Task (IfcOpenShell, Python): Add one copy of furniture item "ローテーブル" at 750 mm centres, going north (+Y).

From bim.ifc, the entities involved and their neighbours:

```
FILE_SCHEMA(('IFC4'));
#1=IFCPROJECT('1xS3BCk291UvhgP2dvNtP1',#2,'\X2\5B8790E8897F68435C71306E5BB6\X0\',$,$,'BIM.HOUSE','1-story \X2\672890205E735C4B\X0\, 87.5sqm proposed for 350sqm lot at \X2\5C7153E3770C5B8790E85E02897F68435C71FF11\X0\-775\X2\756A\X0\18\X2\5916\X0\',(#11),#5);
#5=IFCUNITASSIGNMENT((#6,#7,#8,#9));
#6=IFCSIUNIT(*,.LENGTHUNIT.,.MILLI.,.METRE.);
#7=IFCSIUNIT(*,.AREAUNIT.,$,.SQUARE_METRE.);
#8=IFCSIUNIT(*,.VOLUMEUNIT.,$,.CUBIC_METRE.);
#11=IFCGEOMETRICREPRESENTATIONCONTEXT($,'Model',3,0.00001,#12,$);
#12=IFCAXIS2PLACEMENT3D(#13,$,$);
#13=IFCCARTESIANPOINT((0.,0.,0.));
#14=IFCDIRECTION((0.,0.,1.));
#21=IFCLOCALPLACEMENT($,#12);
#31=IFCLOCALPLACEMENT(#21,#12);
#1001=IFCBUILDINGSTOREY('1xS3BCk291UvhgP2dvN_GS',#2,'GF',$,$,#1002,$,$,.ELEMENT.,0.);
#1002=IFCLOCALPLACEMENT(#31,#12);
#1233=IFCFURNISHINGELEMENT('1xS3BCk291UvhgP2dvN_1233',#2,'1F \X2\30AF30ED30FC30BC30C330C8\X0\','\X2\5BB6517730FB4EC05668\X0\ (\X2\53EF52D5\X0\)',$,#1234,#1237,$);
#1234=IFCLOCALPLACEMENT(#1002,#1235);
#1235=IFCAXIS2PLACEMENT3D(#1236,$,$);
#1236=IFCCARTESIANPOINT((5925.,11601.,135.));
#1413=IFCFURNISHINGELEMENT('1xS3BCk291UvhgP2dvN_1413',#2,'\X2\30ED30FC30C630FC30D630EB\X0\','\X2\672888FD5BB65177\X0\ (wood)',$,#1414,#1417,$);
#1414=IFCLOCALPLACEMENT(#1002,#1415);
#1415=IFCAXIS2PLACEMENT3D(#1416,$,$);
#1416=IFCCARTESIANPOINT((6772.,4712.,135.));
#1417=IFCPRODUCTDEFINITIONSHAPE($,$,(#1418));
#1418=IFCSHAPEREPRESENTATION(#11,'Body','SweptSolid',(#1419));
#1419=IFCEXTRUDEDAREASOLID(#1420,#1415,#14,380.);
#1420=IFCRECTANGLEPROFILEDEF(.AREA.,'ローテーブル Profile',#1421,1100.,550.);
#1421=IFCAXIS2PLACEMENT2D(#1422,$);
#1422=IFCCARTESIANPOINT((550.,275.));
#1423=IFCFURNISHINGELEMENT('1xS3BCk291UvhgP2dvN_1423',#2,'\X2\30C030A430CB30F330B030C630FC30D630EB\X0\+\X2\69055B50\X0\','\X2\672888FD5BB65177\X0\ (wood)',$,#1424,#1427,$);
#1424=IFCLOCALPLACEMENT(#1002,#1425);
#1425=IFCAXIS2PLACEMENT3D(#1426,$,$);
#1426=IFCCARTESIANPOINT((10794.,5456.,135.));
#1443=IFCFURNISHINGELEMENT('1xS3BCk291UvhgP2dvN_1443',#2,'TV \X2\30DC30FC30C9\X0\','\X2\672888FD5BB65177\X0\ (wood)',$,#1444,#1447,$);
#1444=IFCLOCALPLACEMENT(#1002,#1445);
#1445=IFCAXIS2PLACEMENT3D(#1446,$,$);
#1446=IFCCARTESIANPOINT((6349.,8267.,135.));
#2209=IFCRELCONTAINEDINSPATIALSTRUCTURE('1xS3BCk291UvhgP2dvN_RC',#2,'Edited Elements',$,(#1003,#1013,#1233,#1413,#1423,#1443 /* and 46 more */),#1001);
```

```python
import numpy as np
import ifcopenshell
import ifcopenshell.api.geometry
import ifcopenshell.api.root
import ifcopenshell.util.element
import ifcopenshell.util.placement

model = ifcopenshell.open("bim.ifc")


def reuse_history(source, copy):
    """copy_class also copies each property set's owner history, people and application; keep the originals."""
    for rel in copy.IsDefinedBy:
        if rel.is_a("IfcRelDefinesByProperties") and (history := rel.RelatingPropertyDefinition.OwnerHistory):
            rel.RelatingPropertyDefinition.OwnerHistory = source.OwnerHistory
            ifcopenshell.util.element.remove_deep2(model, history)


source = model.by_id(1413)
base = ifcopenshell.util.placement.get_local_placement(source.ObjectPlacement)
step = np.array([0.0, 1.0, 0.0]) * 750.0

for i in range(1, 2):
    copy = ifcopenshell.api.root.copy_class(model, product=source)
    copy.Representation = ifcopenshell.util.element.copy_deep(
        model, source.Representation, exclude=["IfcGeometricRepresentationContext", "IfcRepresentationMap"]
    )
    reuse_history(source, copy)
    matrix = base.copy()
    matrix[:3, 3] += i * step
    print("added at", matrix[:3, 3].round(3) + 0.0)
    ifcopenshell.api.geometry.edit_object_placement(model, product=copy, matrix=matrix, is_si=False)

model.write("bim-out.ifc")
```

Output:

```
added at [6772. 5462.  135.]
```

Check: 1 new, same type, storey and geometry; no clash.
